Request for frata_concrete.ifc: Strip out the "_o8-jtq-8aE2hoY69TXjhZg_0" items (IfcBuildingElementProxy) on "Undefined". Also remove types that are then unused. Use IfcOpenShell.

First a look at what the model holds.

```python
import ifcopenshell
import ifcopenshell.util.element

model = ifcopenshell.open("frata_concrete.ifc")
print(model.schema)
storey = next(s for s in model.by_type("IfcBuildingStorey") if s.Name == "Undefined")
proxies = [e for e in ifcopenshell.util.element.get_decomposition(storey) if e.is_a("IfcBuildingElementProxy")]
seen = {}
for e in proxies:
    element_type = ifcopenshell.util.element.get_type(e)
    name = element_type.Name if element_type not in (None, e) else None
    seen[name] = seen.get(name, 0) + 1
for name, count in sorted(seen.items(), key=str):
    print(count, "x", name)
```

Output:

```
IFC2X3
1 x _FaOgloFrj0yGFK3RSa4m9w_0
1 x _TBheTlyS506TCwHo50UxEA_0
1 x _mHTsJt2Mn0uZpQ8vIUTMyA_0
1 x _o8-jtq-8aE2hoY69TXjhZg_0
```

```python
import ifcopenshell
import ifcopenshell.api.root
import ifcopenshell.util.element

model = ifcopenshell.open("frata_concrete.ifc")

storey = next(s for s in model.by_type("IfcBuildingStorey") if s.Name == "Undefined")
proxies = [e for e in ifcopenshell.util.element.get_decomposition(storey) if e.is_a("IfcBuildingElementProxy")]
targets = [e for e in proxies if (t := ifcopenshell.util.element.get_type(e)) not in (None, e) and t.Name == "_o8-jtq-8aE2hoY69TXjhZg_0"]
types = {ifcopenshell.util.element.get_type(e) for e in targets} - {None, *targets}

for e in targets:
    ifcopenshell.api.root.remove_product(model, product=e)
print(len(targets), "removed")

unused = [t for t in types if not ifcopenshell.util.element.get_types(t)]
for t in unused:
    ifcopenshell.api.root.remove_product(model, product=t)
print(len(unused), "unused types removed")

model.write("frata_concrete_rev.ifc")
```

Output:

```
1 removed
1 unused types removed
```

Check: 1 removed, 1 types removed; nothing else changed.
